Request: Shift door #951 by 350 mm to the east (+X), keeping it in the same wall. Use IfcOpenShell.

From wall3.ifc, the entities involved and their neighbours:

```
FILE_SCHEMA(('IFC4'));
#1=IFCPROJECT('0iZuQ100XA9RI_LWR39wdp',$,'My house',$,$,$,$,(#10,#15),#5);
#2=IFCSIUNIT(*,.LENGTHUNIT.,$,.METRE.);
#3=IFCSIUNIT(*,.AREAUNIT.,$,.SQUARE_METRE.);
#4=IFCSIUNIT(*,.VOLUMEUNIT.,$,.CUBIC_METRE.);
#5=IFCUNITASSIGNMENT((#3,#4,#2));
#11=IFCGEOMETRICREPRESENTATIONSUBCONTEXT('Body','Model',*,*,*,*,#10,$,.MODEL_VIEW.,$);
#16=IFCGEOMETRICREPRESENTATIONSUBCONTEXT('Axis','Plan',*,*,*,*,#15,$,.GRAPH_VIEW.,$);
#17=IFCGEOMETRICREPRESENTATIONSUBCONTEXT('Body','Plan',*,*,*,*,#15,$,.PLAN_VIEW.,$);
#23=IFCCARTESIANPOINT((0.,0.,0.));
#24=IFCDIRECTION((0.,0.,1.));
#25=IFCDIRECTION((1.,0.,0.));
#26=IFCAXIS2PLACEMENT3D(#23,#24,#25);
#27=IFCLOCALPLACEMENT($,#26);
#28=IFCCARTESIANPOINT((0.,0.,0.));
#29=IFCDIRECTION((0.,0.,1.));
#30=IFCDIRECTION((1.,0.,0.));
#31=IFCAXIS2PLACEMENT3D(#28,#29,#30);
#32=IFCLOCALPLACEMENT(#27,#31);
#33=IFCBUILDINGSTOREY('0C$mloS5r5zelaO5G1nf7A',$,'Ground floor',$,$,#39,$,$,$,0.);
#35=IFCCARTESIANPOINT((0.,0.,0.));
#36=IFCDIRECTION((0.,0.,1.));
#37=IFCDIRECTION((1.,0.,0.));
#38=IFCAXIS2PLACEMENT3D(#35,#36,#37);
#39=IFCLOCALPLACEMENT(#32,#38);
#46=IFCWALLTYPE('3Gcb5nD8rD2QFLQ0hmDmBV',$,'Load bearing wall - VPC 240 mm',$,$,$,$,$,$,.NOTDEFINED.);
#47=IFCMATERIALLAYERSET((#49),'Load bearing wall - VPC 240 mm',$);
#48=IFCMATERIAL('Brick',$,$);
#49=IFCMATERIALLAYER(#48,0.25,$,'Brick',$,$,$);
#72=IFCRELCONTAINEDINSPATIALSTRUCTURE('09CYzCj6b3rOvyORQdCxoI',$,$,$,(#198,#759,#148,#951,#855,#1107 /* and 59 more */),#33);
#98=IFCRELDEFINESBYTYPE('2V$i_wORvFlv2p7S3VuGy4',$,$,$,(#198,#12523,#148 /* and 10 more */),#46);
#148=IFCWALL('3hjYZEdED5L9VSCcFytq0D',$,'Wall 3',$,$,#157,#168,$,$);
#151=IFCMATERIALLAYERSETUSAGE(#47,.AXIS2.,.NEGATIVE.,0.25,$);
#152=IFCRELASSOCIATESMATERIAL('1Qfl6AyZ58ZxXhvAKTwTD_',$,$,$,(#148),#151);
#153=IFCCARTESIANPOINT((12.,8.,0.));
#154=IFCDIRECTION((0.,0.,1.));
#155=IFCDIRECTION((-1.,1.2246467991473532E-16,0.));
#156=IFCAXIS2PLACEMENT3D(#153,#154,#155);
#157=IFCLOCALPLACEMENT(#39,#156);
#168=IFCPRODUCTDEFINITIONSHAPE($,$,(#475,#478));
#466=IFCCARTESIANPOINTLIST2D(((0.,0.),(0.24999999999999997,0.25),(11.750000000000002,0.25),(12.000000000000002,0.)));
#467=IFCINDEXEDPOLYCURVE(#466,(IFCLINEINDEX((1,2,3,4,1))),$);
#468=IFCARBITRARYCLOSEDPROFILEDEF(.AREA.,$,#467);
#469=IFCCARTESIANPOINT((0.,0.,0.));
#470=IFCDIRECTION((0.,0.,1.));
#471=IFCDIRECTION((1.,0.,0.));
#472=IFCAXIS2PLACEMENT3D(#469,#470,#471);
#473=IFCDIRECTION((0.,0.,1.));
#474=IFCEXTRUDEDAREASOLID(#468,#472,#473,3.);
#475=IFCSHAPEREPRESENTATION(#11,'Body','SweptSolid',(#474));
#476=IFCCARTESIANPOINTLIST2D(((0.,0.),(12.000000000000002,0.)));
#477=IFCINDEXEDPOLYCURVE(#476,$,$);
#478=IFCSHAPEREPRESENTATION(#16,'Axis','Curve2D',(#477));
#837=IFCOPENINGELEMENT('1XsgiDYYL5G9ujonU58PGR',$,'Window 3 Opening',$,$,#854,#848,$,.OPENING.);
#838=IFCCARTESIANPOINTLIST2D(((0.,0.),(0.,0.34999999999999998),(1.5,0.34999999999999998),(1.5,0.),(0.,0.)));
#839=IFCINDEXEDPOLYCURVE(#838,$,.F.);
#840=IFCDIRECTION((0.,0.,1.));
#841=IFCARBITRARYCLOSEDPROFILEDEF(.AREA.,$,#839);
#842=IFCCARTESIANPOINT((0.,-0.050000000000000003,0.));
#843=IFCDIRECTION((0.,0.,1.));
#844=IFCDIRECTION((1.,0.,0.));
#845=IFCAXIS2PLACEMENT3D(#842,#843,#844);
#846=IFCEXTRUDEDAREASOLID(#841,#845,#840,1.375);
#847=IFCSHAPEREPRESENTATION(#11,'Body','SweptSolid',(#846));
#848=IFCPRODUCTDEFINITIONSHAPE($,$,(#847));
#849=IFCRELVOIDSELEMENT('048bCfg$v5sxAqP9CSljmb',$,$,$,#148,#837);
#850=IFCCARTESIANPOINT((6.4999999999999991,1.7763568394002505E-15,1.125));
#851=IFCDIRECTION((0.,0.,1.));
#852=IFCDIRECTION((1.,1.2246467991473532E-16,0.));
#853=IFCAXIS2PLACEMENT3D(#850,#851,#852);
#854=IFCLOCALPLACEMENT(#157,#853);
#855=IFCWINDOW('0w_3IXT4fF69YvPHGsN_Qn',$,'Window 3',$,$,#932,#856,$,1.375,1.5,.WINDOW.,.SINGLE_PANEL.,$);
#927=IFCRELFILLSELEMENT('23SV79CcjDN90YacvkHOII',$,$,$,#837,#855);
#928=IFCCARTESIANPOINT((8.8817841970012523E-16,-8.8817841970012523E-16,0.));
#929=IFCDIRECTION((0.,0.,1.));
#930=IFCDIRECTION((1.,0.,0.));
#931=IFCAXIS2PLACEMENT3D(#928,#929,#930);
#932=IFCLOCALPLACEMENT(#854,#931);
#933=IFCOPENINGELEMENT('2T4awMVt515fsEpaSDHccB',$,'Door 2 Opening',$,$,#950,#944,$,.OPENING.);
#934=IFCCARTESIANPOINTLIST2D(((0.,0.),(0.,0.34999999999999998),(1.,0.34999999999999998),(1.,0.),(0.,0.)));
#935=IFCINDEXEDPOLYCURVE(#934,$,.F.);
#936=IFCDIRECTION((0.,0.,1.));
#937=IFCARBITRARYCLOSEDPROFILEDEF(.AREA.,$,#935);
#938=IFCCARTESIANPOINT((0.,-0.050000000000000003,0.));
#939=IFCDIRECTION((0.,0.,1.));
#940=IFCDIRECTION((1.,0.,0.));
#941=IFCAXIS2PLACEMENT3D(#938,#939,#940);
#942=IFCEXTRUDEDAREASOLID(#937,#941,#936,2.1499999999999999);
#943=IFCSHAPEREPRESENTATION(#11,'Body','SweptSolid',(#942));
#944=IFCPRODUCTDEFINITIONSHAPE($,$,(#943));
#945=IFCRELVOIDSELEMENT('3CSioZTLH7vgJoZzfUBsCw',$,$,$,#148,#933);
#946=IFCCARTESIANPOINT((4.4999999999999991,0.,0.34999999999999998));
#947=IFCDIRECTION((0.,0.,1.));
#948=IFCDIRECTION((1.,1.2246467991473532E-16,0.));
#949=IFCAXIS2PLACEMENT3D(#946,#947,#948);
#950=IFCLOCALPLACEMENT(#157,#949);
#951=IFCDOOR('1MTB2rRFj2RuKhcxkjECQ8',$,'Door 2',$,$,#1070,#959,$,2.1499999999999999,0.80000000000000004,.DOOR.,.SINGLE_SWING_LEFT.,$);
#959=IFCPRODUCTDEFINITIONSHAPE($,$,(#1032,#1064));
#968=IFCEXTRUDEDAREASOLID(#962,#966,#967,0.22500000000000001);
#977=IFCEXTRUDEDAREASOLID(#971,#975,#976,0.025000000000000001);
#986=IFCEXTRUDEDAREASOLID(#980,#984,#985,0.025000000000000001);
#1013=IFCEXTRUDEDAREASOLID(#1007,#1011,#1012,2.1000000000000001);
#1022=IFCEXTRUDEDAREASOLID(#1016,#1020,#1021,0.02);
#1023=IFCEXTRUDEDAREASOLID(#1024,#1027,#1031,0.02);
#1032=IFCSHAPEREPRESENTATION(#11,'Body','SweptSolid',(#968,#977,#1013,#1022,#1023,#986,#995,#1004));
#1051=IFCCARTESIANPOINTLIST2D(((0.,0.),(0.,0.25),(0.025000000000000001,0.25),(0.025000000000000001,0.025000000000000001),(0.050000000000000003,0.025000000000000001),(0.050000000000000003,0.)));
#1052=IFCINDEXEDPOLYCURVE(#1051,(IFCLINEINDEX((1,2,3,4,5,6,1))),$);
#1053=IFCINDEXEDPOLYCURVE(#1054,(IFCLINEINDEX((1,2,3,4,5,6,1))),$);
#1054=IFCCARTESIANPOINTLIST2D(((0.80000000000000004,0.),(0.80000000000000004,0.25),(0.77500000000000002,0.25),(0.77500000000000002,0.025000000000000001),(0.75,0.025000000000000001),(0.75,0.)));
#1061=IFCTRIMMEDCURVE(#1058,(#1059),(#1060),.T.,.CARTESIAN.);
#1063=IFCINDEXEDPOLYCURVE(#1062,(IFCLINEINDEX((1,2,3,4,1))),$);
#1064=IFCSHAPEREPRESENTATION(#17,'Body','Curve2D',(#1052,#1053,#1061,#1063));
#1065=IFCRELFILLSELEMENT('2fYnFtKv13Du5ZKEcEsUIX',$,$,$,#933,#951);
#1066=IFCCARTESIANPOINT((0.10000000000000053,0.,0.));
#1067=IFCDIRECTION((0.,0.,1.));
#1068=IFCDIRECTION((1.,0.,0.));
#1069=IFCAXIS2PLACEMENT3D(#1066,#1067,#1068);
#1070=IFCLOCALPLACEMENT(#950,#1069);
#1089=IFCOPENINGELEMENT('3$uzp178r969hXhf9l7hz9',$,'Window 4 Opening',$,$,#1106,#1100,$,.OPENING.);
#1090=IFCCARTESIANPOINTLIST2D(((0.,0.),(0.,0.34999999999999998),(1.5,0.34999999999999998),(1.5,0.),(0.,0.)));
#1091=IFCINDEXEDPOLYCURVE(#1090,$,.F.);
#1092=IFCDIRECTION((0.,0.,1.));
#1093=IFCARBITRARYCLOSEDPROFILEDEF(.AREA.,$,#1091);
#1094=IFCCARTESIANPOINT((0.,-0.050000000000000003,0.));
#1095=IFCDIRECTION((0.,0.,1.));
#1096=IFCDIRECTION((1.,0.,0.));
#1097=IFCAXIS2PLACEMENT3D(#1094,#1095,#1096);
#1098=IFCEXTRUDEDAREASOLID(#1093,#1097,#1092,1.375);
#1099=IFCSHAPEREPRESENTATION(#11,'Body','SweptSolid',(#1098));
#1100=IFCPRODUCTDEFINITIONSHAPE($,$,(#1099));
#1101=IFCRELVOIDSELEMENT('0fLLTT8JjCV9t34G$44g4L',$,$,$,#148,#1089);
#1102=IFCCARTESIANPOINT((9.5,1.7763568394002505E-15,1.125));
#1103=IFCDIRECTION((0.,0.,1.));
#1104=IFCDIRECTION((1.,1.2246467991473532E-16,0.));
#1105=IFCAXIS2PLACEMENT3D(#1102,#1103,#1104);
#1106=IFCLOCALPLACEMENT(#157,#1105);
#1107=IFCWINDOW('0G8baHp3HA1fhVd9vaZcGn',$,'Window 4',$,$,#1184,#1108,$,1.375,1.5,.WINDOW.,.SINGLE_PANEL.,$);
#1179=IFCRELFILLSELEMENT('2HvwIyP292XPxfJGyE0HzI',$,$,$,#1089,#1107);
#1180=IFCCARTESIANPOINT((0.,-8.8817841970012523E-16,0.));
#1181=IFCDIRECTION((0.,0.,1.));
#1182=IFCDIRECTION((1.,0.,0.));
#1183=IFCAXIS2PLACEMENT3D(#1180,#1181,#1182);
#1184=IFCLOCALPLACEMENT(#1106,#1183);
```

```python
import ifcopenshell
import ifcopenshell.api.geometry
import ifcopenshell.util.placement
import ifcopenshell.util.unit

model = ifcopenshell.open("wall3.ifc")
unit_scale = ifcopenshell.util.unit.calculate_unit_scale(model)

door = model.by_id(951)
opening = door.FillsVoids[0].RelatingOpeningElement
wall = opening.VoidsElements[0].RelatingBuildingElement

wall_matrix = ifcopenshell.util.placement.get_local_placement(wall.ObjectPlacement)
shift = wall_matrix[:3, 0] * -0.35 / unit_scale
before = ifcopenshell.util.placement.get_local_placement(door.ObjectPlacement)[:3, 3].copy()

# The door is placed relative to its opening, so it follows when the opening moves.
matrix = ifcopenshell.util.placement.get_local_placement(opening.ObjectPlacement)
matrix[:3, 3] += shift
ifcopenshell.api.geometry.edit_object_placement(
    model, product=opening, matrix=matrix, is_si=False, should_transform_children=True
)

after = ifcopenshell.util.placement.get_local_placement(door.ObjectPlacement)[:3, 3]
print("door moved by", (after - before).round(3) + 0.0)

model.write("wall3_edited.ifc")
```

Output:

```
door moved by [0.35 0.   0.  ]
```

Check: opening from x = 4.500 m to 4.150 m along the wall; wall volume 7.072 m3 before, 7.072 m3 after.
